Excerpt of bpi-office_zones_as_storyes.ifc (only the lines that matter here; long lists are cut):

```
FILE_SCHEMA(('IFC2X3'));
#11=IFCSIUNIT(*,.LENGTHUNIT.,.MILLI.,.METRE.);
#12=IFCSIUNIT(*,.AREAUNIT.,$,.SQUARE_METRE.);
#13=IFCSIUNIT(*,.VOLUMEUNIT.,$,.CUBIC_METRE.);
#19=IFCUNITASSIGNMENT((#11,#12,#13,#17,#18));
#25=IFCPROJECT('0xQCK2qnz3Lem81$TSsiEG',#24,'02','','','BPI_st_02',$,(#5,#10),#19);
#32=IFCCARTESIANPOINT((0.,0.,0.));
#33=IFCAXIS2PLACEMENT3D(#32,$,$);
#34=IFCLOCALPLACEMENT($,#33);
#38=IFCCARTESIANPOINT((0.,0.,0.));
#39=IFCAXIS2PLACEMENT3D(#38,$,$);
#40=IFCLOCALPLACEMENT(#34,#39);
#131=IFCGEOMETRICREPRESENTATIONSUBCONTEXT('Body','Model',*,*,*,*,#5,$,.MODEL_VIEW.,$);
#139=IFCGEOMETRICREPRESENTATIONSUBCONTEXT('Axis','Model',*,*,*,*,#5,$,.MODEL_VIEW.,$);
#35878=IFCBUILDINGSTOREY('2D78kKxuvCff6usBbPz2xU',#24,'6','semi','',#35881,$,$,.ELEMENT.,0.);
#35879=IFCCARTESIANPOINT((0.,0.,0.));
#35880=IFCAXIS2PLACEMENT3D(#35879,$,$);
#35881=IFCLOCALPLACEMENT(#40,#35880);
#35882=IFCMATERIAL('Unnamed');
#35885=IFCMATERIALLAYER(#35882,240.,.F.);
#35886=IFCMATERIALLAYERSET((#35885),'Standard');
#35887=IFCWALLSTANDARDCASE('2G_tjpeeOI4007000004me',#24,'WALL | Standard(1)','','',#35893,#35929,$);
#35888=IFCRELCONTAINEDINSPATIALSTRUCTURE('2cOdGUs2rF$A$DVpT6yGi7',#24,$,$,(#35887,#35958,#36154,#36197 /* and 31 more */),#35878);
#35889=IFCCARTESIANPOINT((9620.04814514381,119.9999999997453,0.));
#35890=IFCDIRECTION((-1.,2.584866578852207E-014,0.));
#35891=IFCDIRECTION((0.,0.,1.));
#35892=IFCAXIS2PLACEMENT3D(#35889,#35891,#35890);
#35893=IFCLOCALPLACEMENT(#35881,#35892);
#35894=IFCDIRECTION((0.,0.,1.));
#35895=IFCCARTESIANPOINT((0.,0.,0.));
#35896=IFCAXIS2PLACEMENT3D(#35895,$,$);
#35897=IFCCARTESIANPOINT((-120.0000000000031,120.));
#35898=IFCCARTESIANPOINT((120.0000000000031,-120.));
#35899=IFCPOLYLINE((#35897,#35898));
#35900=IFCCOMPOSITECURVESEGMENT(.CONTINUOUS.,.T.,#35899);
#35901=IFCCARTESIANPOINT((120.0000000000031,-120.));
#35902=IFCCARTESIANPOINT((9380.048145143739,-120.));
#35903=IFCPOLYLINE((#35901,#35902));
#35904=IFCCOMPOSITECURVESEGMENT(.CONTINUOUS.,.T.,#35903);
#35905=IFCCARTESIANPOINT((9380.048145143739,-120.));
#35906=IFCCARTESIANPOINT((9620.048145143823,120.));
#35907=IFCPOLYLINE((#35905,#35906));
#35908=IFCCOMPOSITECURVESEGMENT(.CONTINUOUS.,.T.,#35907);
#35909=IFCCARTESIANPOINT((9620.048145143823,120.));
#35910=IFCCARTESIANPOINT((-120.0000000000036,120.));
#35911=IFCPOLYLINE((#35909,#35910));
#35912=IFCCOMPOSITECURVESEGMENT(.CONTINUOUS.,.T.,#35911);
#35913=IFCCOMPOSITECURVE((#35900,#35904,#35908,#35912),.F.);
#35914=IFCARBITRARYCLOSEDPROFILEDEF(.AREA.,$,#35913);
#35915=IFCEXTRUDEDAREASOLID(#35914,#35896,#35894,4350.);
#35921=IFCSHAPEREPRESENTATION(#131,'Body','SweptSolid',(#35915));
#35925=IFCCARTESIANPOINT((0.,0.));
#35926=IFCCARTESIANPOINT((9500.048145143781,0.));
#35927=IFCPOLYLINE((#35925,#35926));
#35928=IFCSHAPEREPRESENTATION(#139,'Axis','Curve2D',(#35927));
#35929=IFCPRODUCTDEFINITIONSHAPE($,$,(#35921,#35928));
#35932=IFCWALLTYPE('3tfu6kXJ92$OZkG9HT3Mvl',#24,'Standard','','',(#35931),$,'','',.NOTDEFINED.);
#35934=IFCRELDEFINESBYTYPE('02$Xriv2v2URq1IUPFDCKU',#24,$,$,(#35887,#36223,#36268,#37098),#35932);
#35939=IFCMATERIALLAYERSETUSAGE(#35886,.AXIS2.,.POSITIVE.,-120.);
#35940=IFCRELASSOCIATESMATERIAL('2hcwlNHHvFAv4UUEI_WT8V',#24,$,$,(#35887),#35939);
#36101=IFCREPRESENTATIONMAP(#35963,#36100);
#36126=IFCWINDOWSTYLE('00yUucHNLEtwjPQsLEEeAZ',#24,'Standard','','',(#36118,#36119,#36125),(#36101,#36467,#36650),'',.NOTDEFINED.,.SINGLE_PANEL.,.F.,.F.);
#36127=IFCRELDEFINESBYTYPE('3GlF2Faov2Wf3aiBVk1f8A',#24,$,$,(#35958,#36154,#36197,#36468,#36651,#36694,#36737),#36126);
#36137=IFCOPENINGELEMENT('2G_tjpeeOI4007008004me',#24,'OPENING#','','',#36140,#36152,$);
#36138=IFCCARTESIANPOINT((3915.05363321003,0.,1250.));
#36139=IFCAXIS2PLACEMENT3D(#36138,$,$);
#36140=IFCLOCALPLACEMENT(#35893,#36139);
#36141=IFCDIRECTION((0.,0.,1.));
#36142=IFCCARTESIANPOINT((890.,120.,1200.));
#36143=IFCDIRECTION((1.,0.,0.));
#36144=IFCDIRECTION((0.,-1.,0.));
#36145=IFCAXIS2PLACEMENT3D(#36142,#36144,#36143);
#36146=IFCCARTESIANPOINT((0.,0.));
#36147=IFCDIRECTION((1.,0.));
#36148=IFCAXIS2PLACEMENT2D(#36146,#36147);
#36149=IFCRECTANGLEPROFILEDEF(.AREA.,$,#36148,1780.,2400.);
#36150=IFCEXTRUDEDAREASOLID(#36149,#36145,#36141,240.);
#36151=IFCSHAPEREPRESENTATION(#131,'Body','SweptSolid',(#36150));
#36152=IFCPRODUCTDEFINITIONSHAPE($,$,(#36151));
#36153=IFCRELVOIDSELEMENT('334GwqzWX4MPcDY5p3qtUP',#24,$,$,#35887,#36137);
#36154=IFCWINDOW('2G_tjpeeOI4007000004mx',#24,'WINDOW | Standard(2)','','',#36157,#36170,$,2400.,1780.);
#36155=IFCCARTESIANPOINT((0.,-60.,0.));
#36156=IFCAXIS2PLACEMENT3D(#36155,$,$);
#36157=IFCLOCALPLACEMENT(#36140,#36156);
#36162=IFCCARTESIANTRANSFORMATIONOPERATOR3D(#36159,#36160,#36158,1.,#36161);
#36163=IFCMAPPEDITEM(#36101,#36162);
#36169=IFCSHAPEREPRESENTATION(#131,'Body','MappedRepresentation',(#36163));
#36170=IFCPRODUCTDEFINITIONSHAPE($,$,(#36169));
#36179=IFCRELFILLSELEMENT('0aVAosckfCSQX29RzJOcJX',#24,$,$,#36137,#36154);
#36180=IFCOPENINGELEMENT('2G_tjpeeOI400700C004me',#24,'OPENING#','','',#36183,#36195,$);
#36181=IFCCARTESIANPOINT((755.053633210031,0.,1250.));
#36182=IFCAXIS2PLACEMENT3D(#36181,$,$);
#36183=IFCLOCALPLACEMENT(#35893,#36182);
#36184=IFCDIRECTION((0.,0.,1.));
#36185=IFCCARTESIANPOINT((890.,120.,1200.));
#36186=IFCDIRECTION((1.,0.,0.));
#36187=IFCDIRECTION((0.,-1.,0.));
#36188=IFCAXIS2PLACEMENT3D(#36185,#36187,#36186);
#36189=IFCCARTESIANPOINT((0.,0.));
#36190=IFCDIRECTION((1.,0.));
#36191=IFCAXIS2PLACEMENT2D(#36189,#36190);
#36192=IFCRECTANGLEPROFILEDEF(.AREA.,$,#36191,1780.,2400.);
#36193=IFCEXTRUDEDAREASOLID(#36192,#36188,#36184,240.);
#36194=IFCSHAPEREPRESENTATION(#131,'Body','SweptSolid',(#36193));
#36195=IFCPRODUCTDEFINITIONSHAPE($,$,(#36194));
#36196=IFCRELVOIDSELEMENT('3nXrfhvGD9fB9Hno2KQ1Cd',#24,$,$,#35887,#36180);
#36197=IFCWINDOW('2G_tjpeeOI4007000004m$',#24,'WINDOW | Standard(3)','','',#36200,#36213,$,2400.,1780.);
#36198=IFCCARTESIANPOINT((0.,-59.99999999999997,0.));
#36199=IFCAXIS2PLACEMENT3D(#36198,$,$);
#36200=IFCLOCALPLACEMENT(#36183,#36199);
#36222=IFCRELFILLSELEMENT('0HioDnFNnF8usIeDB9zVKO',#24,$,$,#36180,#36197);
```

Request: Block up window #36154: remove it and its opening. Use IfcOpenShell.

```python
import ifcopenshell
import ifcopenshell.api.feature
import ifcopenshell.api.root
import ifcopenshell.geom
import ifcopenshell.util.shape

model = ifcopenshell.open("bpi-office_zones_as_storyes.ifc")
settings = ifcopenshell.geom.settings()


def volume(element):
    """Net volume in cubic metres, openings subtracted."""
    shape = ifcopenshell.geom.create_shape(settings, element)
    return ifcopenshell.util.shape.get_volume(shape.geometry)


window = model.by_guid("2G_tjpeeOI4007000004mx")
opening = window.FillsVoids[0].RelatingOpeningElement
wall = opening.VoidsElements[0].RelatingBuildingElement
before = volume(wall)

ifcopenshell.api.root.remove_product(model, product=window)
ifcopenshell.api.feature.remove_feature(model, feature=opening)

after = volume(wall)

print(f"wall volume {before:.3f} -> {after:.3f} m3")

model.write("bpi-office_zones_as_storyes_rev.ifc")
```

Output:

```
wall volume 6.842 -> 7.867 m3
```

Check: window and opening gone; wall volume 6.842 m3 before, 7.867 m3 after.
